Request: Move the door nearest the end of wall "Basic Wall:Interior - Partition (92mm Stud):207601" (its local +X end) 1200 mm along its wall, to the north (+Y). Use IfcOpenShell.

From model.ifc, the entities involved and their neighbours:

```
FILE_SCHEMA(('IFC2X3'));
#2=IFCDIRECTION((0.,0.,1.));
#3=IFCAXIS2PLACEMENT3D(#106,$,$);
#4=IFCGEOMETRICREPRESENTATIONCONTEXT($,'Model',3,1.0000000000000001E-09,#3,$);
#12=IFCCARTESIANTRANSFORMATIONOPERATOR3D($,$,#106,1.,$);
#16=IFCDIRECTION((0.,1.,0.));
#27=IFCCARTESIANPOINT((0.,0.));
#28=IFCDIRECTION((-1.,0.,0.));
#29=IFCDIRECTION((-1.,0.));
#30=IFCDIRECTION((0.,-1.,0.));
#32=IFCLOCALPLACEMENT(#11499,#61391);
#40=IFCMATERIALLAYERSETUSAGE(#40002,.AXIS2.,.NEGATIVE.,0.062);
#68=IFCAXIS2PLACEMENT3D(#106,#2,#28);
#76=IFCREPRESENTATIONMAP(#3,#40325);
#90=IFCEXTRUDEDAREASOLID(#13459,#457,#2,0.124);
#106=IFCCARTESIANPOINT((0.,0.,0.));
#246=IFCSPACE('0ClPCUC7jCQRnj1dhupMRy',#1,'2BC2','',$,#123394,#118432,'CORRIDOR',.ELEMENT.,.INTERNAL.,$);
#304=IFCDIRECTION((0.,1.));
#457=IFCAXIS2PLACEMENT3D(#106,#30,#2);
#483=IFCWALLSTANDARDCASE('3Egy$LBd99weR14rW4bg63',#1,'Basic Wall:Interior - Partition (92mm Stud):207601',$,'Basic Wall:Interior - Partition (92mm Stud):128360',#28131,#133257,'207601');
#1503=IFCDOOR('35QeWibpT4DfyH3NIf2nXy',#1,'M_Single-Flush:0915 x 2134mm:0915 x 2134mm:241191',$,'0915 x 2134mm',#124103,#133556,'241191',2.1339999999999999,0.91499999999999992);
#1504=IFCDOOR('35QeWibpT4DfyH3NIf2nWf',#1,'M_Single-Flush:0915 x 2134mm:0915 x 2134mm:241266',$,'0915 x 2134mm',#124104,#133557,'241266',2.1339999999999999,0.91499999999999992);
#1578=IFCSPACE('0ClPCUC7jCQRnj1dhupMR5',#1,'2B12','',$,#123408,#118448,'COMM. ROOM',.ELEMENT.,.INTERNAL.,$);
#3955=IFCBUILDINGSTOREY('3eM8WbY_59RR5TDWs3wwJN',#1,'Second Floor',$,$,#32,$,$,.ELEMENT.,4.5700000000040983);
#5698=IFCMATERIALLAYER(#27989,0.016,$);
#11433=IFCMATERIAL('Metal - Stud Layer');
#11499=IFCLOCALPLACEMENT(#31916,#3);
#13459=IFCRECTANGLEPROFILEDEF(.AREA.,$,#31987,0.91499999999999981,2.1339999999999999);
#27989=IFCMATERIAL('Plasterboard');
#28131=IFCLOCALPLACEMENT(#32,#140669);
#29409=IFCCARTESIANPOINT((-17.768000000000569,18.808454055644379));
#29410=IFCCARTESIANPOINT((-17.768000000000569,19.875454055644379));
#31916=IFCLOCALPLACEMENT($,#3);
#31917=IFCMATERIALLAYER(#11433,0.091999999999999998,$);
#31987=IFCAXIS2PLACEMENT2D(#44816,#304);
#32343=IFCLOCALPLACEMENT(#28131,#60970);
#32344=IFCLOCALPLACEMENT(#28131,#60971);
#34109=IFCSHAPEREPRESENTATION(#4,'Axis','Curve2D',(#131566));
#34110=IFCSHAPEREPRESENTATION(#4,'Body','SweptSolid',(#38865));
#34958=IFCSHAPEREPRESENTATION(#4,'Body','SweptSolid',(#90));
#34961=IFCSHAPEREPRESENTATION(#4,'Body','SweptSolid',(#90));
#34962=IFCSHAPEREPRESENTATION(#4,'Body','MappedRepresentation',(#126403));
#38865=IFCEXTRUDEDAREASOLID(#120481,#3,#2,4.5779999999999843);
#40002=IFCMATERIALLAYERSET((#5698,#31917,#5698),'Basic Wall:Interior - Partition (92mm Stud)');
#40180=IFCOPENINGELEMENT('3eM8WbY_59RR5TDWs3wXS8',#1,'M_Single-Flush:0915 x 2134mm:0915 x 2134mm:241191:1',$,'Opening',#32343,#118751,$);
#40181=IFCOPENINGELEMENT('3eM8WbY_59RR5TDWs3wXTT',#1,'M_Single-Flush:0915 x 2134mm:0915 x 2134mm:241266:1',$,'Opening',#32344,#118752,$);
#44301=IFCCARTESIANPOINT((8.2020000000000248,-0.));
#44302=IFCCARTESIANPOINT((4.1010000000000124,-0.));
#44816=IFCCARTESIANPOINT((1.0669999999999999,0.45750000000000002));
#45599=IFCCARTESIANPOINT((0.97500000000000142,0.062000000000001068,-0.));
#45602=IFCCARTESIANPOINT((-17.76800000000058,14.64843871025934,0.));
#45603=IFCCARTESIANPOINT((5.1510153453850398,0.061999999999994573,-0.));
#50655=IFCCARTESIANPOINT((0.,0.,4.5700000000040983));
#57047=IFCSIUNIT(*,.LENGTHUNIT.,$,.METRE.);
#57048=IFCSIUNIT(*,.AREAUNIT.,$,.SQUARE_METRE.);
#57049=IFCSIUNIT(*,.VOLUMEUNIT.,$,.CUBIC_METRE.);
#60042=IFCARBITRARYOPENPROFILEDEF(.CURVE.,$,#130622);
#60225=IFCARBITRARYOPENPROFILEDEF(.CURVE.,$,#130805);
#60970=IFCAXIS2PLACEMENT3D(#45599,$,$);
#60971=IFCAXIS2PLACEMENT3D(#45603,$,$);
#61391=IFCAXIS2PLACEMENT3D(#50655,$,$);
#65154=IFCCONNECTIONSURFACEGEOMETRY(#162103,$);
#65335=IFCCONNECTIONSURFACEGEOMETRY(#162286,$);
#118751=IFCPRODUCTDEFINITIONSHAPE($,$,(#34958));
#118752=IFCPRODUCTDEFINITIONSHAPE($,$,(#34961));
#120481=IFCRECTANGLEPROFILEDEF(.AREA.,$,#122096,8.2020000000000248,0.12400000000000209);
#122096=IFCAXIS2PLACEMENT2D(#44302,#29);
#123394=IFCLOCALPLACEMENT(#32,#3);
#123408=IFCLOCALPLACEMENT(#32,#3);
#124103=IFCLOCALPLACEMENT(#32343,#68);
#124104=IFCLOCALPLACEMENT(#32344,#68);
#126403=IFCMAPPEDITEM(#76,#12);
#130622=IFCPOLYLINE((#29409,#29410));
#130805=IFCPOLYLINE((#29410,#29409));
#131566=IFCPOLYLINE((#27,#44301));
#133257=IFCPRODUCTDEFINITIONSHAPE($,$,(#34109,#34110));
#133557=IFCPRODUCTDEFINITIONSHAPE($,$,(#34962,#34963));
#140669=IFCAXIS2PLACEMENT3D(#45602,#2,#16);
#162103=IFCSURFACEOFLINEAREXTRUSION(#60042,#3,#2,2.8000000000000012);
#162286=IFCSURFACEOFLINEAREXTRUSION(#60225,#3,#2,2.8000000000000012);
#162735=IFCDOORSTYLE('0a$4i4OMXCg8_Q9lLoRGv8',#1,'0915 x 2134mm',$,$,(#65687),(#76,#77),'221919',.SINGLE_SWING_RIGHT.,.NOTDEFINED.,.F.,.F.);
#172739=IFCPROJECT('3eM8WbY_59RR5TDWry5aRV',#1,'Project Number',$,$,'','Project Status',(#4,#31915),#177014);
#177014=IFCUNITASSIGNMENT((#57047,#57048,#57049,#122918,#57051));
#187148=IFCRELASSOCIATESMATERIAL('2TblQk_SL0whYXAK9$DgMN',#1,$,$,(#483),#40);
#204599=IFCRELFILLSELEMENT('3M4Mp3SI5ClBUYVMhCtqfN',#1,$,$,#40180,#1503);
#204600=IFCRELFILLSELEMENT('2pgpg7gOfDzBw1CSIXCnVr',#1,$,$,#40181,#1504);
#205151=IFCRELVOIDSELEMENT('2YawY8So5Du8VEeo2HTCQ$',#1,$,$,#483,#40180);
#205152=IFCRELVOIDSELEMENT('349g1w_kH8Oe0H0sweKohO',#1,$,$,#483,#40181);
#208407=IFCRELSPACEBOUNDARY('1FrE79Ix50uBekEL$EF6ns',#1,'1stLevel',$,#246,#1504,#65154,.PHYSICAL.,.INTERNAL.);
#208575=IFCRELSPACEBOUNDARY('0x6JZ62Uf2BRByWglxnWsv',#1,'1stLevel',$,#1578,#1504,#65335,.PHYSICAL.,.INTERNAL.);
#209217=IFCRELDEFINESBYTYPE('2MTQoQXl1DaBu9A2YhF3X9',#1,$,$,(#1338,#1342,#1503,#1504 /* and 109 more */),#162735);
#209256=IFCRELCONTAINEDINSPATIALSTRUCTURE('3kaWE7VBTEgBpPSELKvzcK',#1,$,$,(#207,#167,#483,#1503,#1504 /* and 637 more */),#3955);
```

```python
import numpy as np
import ifcopenshell
import ifcopenshell.api.geometry
import ifcopenshell.util.placement
import ifcopenshell.util.unit

model = ifcopenshell.open("model.ifc")
unit_scale = ifcopenshell.util.unit.calculate_unit_scale(model)

door = model.by_guid("35QeWibpT4DfyH3NIf2nWf")
opening = door.FillsVoids[0].RelatingOpeningElement
wall = opening.VoidsElements[0].RelatingBuildingElement

wall_matrix = ifcopenshell.util.placement.get_local_placement(wall.ObjectPlacement)
shift = wall_matrix[:3, 0] * 1.2 / unit_scale
before = ifcopenshell.util.placement.get_local_placement(door.ObjectPlacement)[:3, 3].copy()

# The door is placed relative to its opening, so it follows when the opening moves.
matrix = ifcopenshell.util.placement.get_local_placement(opening.ObjectPlacement)
matrix[:3, 3] += shift
ifcopenshell.api.geometry.edit_object_placement(
    model, product=opening, matrix=matrix, is_si=False, should_transform_children=True
)

# Space boundary surfaces are stored in each space's coordinates; move them too.
for rel in door.ProvidesBoundaries:
    if not rel.ConnectionGeometry:
        continue
    surface = rel.ConnectionGeometry.SurfaceOnRelatingElement
    space_matrix = ifcopenshell.util.placement.get_local_placement(rel.RelatingSpace.ObjectPlacement)
    point = np.array(surface.Position.Location.Coordinates) + space_matrix[:3, :3].T @ shift
    surface.Position = model.createIfcAxis2Placement3D(
        model.createIfcCartesianPoint(point.tolist()), surface.Position.Axis, surface.Position.RefDirection
    )

after = ifcopenshell.util.placement.get_local_placement(door.ObjectPlacement)[:3, 3]
print("door moved by", (after - before).round(3) + 0.0)

model.write("model_updated.ifc")
```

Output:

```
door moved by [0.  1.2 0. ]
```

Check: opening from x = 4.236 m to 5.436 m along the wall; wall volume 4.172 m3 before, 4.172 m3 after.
